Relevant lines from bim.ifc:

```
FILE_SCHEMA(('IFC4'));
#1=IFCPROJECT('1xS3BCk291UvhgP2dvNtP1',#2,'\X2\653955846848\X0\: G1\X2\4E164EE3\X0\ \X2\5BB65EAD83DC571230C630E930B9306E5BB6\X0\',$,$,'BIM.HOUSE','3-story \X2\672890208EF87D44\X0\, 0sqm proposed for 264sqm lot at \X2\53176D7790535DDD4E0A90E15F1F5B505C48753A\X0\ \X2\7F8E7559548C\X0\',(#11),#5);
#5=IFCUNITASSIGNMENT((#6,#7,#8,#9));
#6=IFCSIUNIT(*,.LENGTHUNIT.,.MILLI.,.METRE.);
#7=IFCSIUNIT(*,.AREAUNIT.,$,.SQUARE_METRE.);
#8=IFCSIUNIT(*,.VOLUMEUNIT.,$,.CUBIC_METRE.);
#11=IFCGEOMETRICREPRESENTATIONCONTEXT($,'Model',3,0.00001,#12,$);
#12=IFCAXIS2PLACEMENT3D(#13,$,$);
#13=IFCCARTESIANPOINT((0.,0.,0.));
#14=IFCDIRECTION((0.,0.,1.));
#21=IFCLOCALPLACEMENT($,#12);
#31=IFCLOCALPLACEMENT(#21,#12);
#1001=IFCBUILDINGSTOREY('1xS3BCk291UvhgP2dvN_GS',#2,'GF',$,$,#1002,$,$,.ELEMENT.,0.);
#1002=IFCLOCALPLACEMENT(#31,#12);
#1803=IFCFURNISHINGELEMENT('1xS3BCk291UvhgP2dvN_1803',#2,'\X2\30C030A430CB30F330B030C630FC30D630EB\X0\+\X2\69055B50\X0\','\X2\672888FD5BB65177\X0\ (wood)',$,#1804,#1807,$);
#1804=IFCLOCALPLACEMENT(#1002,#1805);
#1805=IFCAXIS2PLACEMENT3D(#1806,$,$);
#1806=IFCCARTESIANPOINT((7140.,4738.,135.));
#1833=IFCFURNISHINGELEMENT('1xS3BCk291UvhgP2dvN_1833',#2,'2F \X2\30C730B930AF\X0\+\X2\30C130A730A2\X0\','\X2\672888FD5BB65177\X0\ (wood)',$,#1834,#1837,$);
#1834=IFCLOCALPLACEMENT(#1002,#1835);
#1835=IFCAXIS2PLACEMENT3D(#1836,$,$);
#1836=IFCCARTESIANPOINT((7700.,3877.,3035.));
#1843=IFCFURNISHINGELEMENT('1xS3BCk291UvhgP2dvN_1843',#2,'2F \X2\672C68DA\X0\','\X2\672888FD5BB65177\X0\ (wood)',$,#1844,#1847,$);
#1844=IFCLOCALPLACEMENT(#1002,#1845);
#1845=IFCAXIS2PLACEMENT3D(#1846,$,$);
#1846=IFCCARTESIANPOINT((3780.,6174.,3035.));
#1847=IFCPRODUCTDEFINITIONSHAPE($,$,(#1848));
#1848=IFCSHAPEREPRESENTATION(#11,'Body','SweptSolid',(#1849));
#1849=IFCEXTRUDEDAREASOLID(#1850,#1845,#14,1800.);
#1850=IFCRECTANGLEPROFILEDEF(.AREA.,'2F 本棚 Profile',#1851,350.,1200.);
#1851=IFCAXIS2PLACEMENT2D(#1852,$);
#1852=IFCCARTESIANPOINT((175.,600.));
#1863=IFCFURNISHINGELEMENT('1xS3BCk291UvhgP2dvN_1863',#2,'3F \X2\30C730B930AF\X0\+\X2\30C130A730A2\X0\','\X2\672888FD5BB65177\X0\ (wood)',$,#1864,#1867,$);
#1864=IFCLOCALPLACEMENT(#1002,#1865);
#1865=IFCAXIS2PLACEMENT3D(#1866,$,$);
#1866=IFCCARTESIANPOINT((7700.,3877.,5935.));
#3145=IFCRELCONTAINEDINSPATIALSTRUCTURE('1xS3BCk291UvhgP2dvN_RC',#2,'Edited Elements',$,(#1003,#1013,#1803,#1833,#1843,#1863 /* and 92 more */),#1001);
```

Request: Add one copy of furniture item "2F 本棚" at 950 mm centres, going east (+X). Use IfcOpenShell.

```python
import numpy as np
import ifcopenshell
import ifcopenshell.api.geometry
import ifcopenshell.api.root
import ifcopenshell.util.element
import ifcopenshell.util.placement
import ifcopenshell.util.unit

model = ifcopenshell.open("bim.ifc")
unit_scale = ifcopenshell.util.unit.calculate_unit_scale(model)


def reuse_history(source, copy):
    """copy_class also copies each property set's owner history, people and application; keep the originals."""
    for rel in copy.IsDefinedBy:
        if rel.is_a("IfcRelDefinesByProperties") and (history := rel.RelatingPropertyDefinition.OwnerHistory):
            rel.RelatingPropertyDefinition.OwnerHistory = source.OwnerHistory
            ifcopenshell.util.element.remove_deep2(model, history)


source = model.by_guid("1xS3BCk291UvhgP2dvN_1843")
base = ifcopenshell.util.placement.get_local_placement(source.ObjectPlacement)
step = np.array([1.0, 0.0, 0.0]) * 0.95 / unit_scale

for i in range(1, 2):
    copy = ifcopenshell.api.root.copy_class(model, product=source)
    copy.Representation = ifcopenshell.util.element.copy_deep(
        model, source.Representation, exclude=["IfcGeometricRepresentationContext", "IfcRepresentationMap"]
    )
    reuse_history(source, copy)
    matrix = base.copy()
    matrix[:3, 3] += i * step
    print("added at", matrix[:3, 3].round(3) + 0.0)
    ifcopenshell.api.geometry.edit_object_placement(model, product=copy, matrix=matrix, is_si=False)

model.write("bim_updated.ifc")
```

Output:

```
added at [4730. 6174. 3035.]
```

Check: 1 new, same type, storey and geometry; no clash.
